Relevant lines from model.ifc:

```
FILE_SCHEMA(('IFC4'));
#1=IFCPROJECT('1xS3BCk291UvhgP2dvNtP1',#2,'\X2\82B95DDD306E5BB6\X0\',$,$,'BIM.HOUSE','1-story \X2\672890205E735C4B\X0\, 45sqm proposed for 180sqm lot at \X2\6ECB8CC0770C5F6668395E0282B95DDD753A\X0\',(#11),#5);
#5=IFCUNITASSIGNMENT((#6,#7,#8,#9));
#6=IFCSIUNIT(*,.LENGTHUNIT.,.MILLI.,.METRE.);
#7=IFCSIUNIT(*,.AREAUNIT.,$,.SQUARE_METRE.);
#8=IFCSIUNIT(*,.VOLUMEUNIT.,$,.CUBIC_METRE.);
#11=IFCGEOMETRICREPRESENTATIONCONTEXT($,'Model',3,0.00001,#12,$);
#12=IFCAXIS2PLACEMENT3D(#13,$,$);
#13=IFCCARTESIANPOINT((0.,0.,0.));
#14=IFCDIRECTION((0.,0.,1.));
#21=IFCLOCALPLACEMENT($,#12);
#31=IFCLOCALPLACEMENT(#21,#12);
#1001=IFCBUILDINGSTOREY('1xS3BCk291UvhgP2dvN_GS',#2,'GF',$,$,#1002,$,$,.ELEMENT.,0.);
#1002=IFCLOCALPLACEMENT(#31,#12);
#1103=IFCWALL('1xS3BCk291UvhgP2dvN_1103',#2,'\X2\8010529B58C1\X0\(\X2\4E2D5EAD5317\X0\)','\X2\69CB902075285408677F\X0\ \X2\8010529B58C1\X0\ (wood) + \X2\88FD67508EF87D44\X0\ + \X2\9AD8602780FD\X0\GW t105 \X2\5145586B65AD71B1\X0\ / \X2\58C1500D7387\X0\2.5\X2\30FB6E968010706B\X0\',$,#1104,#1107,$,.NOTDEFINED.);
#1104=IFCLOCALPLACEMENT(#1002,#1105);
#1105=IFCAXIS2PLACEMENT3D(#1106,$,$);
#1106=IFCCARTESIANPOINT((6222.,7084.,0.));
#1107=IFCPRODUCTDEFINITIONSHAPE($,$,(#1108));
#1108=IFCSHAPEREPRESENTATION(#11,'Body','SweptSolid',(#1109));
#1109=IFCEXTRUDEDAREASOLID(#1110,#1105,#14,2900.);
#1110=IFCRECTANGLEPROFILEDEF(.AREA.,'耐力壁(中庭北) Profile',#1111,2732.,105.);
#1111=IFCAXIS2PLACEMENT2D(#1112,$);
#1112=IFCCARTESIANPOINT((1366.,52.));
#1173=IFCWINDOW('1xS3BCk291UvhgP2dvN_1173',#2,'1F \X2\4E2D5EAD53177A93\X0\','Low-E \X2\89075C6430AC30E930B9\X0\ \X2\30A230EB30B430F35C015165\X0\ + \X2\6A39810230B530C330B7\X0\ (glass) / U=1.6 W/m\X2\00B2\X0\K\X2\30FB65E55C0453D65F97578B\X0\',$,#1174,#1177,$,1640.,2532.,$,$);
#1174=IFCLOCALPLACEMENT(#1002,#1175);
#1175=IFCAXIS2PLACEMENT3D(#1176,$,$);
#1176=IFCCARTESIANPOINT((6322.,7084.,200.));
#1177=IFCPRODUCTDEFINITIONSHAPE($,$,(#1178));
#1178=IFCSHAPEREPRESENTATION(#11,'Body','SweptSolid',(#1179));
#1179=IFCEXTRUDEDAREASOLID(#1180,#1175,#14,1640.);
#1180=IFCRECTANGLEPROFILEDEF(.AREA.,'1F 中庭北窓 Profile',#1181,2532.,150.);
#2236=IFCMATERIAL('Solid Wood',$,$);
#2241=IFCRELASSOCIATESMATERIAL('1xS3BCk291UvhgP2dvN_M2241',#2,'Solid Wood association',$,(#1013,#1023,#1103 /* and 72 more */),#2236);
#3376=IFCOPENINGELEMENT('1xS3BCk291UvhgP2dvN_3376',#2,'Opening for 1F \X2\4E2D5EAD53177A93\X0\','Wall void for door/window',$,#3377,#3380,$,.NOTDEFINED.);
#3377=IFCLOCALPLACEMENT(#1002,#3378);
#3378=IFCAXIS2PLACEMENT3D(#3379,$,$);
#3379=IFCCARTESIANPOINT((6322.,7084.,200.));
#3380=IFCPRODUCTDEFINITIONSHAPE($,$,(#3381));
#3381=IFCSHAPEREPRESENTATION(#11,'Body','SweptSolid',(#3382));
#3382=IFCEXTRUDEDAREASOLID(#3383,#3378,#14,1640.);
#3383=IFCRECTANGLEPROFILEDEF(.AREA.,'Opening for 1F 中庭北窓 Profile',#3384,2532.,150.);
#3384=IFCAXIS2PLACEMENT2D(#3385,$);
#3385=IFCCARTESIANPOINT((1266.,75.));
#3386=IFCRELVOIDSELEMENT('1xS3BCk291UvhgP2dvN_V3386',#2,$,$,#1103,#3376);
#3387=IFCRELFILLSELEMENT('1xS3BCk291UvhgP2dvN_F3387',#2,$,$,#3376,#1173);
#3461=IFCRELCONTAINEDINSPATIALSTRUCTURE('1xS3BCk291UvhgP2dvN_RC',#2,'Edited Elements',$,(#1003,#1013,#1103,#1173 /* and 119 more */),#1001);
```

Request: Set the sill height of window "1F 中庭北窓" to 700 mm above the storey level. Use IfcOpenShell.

```python
import numpy as np
import ifcopenshell
import ifcopenshell.api.geometry
import ifcopenshell.geom
import ifcopenshell.util.element
import ifcopenshell.util.placement
import ifcopenshell.util.shape
import ifcopenshell.util.unit

model = ifcopenshell.open("model.ifc")
unit_scale = ifcopenshell.util.unit.calculate_unit_scale(model)

window = model.by_id(1173)
opening = window.FillsVoids[0].RelatingOpeningElement
storey = ifcopenshell.util.element.get_container(window, ifc_class="IfcBuildingStorey")
level = ifcopenshell.util.placement.get_local_placement(storey.ObjectPlacement)[2, 3]

# The opening's origin need not be at the sill, so measure its lowest point.
shape = ifcopenshell.geom.create_shape(ifcopenshell.geom.settings(), opening)
bottom = ifcopenshell.util.shape.get_shape_bottom_elevation(shape, shape.geometry) / unit_scale
dz = level + 700.0 - bottom

shift = np.array([0.0, 0.0, dz])
# The window is not placed relative to its opening, so move both.
for product in (opening, window):
    matrix = ifcopenshell.util.placement.get_local_placement(product.ObjectPlacement)
    matrix[:3, 3] += shift
    ifcopenshell.api.geometry.edit_object_placement(model, product=product, matrix=matrix, is_si=False)

print(f"moved by {dz * unit_scale:+.3f} m")

model.write("model_updated.ifc")
```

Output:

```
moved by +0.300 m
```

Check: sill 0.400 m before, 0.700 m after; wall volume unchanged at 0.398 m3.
